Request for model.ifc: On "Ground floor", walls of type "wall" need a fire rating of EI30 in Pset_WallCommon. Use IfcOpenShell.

First a look at what the model holds.

```python
import ifcopenshell
import ifcopenshell.util.element

model = ifcopenshell.open("model.ifc")
print(model.schema)
storey = next(s for s in model.by_type("IfcBuildingStorey") if s.Name == "Ground floor")
walls = [e for e in ifcopenshell.util.element.get_decomposition(storey) if e.is_a("IfcWall")]
seen = {}
for e in walls:
    element_type = ifcopenshell.util.element.get_type(e)
    key = (element_type.Name if element_type != e and element_type else None, ifcopenshell.util.element.get_pset(e, "Pset_WallCommon", "FireRating"))
    seen[key] = seen.get(key, 0) + 1
for (name, value), count in sorted(seen.items(), key=str):
    print(count, "x", name, "|", value)
```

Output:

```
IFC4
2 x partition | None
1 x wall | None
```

```python
import ifcopenshell
import ifcopenshell.api.pset
import ifcopenshell.util.element

model = ifcopenshell.open("model.ifc")

storey = next(s for s in model.by_type("IfcBuildingStorey") if s.Name == "Ground floor")
walls = [e for e in ifcopenshell.util.element.get_decomposition(storey) if e.is_a("IfcWall")]

count = 0
for e in walls:
    element_type = ifcopenshell.util.element.get_type(e)
    if element_type in (None, e) or element_type.Name != "wall":
        continue
    # add_pset returns the element's existing set when there is one.
    pset = ifcopenshell.api.pset.add_pset(model, product=e, name="Pset_WallCommon")
    ifcopenshell.api.pset.edit_pset(model, pset=pset, properties={"FireRating": "EI30"})
    count += 1

print(count, "walls updated")

model.write("model_edited.ifc")
```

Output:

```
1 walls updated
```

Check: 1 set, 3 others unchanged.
